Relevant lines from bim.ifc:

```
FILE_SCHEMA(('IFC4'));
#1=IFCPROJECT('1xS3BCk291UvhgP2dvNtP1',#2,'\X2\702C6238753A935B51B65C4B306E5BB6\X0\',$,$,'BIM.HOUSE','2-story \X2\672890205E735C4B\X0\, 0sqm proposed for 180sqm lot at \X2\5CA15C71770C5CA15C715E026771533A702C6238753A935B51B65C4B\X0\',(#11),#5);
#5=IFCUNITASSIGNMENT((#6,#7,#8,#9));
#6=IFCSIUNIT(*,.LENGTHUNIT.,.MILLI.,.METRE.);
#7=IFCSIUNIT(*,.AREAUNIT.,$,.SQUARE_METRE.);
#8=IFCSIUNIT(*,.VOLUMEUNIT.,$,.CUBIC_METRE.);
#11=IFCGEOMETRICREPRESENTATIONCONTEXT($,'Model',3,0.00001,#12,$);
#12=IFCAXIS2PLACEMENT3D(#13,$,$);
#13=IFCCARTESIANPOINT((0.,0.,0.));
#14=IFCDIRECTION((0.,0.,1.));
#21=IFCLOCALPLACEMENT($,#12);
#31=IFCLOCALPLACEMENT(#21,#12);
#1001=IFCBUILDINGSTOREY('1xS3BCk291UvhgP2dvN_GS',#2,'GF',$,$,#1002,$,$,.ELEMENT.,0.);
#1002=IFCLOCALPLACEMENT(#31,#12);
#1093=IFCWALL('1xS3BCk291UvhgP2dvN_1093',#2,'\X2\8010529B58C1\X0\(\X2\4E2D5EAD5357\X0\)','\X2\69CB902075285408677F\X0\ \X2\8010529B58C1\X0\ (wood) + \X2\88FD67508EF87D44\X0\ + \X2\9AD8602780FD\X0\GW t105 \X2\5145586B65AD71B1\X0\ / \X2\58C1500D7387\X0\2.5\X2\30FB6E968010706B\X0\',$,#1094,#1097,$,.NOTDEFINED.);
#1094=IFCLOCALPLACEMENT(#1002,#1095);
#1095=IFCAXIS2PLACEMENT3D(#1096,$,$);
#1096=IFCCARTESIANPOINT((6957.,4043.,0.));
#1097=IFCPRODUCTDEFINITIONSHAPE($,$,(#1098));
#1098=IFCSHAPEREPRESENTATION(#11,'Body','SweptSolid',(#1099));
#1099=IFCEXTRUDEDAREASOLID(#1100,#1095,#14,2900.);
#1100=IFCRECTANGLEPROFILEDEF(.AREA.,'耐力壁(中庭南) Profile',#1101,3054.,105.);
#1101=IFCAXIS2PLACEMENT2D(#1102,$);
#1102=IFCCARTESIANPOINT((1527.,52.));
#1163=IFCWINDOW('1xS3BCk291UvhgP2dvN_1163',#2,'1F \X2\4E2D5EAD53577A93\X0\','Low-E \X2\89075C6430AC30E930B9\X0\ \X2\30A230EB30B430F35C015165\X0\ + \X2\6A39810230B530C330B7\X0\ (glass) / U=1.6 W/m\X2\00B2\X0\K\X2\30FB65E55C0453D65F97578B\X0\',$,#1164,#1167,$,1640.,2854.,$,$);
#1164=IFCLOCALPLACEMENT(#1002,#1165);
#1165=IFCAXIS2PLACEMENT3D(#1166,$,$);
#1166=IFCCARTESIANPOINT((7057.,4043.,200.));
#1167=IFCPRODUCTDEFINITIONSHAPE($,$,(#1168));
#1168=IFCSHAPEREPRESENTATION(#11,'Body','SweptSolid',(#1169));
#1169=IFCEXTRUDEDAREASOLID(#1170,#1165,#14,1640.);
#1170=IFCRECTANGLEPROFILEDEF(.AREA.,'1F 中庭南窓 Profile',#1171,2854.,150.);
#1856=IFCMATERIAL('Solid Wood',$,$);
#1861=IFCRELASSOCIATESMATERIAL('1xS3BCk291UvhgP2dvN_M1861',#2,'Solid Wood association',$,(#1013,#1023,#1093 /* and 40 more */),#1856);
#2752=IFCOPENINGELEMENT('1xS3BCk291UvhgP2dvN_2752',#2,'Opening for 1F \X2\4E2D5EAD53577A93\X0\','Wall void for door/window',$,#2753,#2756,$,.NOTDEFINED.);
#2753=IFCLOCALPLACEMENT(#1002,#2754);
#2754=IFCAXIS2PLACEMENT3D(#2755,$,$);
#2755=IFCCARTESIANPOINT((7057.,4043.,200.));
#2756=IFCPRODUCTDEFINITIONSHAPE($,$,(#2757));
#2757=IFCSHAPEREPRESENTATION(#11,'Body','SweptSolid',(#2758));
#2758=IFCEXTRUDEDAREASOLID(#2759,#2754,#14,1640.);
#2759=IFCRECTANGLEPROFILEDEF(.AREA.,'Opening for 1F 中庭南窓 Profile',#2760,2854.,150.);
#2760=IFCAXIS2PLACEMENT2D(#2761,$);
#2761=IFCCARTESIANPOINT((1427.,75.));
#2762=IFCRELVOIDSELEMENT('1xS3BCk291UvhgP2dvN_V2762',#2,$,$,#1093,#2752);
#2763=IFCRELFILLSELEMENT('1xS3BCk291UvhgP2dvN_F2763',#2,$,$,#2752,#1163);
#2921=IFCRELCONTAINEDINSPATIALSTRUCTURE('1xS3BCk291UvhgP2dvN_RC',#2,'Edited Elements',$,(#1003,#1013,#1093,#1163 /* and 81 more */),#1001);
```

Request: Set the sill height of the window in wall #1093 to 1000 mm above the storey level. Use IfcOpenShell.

```python
import numpy as np
import ifcopenshell
import ifcopenshell.api.geometry
import ifcopenshell.geom
import ifcopenshell.util.element
import ifcopenshell.util.placement
import ifcopenshell.util.shape
import ifcopenshell.util.unit

model = ifcopenshell.open("bim.ifc")
unit_scale = ifcopenshell.util.unit.calculate_unit_scale(model)

window = model.by_id(1163)
opening = window.FillsVoids[0].RelatingOpeningElement
storey = ifcopenshell.util.element.get_container(window, ifc_class="IfcBuildingStorey")
level = ifcopenshell.util.placement.get_local_placement(storey.ObjectPlacement)[2, 3]

# The opening's origin need not be at the sill, so measure its lowest point.
shape = ifcopenshell.geom.create_shape(ifcopenshell.geom.settings(), opening)
bottom = ifcopenshell.util.shape.get_shape_bottom_elevation(shape, shape.geometry) / unit_scale
dz = level + 1 / unit_scale - bottom

shift = np.array([0.0, 0.0, dz])
# The window is not placed relative to its opening, so move both.
for product in (opening, window):
    matrix = ifcopenshell.util.placement.get_local_placement(product.ObjectPlacement)
    matrix[:3, 3] += shift
    ifcopenshell.api.geometry.edit_object_placement(model, product=product, matrix=matrix, is_si=False)

print(f"moved by {dz * unit_scale:+.3f} m")

model.write("bim_v2.ifc")
```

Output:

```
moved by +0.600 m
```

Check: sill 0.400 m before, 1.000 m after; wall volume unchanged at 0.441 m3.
